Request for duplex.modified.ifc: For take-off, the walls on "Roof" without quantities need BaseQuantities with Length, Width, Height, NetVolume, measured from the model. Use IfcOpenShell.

First a look at what the model holds.

```python
import ifcopenshell
import ifcopenshell.util.element
import ifcopenshell.util.unit

model = ifcopenshell.open("duplex.modified.ifc")
print(model.schema)
for unit_type in ("LENGTHUNIT", "AREAUNIT", "VOLUMEUNIT"):
    print(unit_type, ifcopenshell.util.unit.calculate_unit_scale(model, unit_type))
storey = next(s for s in model.by_type("IfcBuildingStorey") if s.Name == "Roof")
walls = [e for e in ifcopenshell.util.element.get_decomposition(storey) if e.is_a("IfcWall")]
for e in sorted(walls, key=lambda e: e.id()):
    print(e.id(), e.is_a(), e.Name, list(ifcopenshell.util.element.get_psets(e, qtos_only=True)), sep=" | ")
```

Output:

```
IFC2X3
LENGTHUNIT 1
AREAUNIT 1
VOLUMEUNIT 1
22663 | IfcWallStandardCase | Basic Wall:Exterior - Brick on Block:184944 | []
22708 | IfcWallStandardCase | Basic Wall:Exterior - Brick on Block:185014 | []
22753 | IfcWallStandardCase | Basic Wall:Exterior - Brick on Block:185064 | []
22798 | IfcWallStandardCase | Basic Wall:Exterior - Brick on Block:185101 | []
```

```python
import ifcopenshell
import ifcopenshell.api.pset
import ifcopenshell.geom
import ifcopenshell.util.element
import ifcopenshell.util.shape
import ifcopenshell.util.unit

model = ifcopenshell.open("duplex.modified.ifc")
unit_scale = ifcopenshell.util.unit.calculate_unit_scale(model)
volume_scale = ifcopenshell.util.unit.calculate_unit_scale(model, "VOLUMEUNIT")
settings = ifcopenshell.geom.settings()

storey = next(s for s in model.by_type("IfcBuildingStorey") if s.Name == "Roof")
walls = [e for e in ifcopenshell.util.element.get_decomposition(storey) if e.is_a("IfcWall")]

for e in sorted(walls, key=lambda e: e.id()):
    if ifcopenshell.util.element.get_psets(e, qtos_only=True, should_inherit=False):
        continue
    # Geometry comes back in metres, in the element's own axes.
    shape = ifcopenshell.geom.create_shape(settings, e)
    values = {
        "Length": ifcopenshell.util.shape.get_x(shape.geometry) / unit_scale,
        "Width": ifcopenshell.util.shape.get_y(shape.geometry) / unit_scale,
        "Height": ifcopenshell.util.shape.get_z(shape.geometry) / unit_scale,
        "NetVolume": ifcopenshell.util.shape.get_volume(shape.geometry) / volume_scale,
    }
    qto = ifcopenshell.api.pset.add_qto(model, product=e, name="BaseQuantities")
    ifcopenshell.api.pset.edit_qto(model, qto=qto, properties=values)
    print(e.id(), {k: round(v, 3) for k, v in values.items()})

model.write("duplex.modified_edited.ifc")
```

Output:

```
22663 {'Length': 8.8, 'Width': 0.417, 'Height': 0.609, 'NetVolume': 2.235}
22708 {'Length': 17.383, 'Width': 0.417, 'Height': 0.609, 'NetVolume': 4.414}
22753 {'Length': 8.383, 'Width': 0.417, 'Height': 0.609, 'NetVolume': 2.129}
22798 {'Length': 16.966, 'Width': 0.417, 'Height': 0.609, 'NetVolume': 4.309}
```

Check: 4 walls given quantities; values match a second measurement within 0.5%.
